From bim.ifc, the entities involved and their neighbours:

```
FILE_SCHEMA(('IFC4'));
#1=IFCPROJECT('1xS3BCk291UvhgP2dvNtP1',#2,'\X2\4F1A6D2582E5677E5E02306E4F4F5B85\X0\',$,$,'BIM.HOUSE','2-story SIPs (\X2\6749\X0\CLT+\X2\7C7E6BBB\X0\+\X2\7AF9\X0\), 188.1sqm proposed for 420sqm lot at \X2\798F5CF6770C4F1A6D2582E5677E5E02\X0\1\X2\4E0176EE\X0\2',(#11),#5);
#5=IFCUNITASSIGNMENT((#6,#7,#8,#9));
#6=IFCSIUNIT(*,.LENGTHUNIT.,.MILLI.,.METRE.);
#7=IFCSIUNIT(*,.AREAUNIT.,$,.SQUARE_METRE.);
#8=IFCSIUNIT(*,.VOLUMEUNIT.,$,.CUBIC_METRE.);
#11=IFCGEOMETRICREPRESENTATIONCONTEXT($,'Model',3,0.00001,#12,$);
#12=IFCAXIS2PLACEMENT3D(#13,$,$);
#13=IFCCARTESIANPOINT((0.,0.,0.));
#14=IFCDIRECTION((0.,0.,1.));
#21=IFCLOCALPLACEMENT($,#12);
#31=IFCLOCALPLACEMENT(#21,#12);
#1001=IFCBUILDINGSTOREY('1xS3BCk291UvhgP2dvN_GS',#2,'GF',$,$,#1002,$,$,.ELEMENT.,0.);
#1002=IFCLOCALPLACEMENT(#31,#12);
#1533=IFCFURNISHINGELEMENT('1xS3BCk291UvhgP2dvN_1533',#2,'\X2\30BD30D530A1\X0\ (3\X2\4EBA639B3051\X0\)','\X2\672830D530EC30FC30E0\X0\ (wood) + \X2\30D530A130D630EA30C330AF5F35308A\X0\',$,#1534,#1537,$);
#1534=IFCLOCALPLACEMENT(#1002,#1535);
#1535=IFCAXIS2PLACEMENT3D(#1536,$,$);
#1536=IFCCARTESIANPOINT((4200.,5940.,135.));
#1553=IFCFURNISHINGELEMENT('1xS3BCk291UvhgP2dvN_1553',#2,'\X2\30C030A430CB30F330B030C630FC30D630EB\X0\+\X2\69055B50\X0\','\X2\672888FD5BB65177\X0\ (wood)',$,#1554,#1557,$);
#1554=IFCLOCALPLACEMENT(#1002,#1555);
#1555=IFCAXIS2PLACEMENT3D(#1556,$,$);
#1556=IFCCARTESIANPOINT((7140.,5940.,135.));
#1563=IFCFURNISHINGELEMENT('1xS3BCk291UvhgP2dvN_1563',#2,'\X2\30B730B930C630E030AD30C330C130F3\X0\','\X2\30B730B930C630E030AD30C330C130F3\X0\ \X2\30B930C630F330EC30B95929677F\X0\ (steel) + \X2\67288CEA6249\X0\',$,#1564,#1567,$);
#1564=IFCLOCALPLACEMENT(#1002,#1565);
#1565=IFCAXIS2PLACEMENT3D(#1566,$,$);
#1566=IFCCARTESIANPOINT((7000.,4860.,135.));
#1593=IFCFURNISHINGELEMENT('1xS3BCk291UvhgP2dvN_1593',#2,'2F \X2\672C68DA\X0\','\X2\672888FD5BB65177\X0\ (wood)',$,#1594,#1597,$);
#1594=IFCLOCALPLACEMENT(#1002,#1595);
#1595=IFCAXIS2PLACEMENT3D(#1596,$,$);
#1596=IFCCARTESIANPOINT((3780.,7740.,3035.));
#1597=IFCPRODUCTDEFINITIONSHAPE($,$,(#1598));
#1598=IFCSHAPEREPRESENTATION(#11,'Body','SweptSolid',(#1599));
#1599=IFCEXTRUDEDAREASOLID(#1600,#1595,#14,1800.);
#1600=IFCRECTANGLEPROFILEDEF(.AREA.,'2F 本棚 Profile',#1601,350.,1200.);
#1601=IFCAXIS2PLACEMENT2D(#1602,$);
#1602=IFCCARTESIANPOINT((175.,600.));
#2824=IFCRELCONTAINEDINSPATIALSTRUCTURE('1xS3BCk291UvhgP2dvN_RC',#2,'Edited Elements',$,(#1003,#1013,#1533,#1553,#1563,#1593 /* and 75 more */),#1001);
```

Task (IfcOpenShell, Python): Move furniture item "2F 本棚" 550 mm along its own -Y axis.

```python
import ifcopenshell
import ifcopenshell.api.geometry
import ifcopenshell.util.placement

model = ifcopenshell.open("bim.ifc")

item = model.by_id(1593)
matrix = ifcopenshell.util.placement.get_local_placement(item.ObjectPlacement)
matrix[:3, 3] -= matrix[:3, 1] * 550.0
ifcopenshell.api.geometry.edit_object_placement(model, product=item, matrix=matrix, is_si=False)

print(ifcopenshell.util.placement.get_local_placement(item.ObjectPlacement).round(3) + 0.0)

model.write("bim_v2.ifc")
```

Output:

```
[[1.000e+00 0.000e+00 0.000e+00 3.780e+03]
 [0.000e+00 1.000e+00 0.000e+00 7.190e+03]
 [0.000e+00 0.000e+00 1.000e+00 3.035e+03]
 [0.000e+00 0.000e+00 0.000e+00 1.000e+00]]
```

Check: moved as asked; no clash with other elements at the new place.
